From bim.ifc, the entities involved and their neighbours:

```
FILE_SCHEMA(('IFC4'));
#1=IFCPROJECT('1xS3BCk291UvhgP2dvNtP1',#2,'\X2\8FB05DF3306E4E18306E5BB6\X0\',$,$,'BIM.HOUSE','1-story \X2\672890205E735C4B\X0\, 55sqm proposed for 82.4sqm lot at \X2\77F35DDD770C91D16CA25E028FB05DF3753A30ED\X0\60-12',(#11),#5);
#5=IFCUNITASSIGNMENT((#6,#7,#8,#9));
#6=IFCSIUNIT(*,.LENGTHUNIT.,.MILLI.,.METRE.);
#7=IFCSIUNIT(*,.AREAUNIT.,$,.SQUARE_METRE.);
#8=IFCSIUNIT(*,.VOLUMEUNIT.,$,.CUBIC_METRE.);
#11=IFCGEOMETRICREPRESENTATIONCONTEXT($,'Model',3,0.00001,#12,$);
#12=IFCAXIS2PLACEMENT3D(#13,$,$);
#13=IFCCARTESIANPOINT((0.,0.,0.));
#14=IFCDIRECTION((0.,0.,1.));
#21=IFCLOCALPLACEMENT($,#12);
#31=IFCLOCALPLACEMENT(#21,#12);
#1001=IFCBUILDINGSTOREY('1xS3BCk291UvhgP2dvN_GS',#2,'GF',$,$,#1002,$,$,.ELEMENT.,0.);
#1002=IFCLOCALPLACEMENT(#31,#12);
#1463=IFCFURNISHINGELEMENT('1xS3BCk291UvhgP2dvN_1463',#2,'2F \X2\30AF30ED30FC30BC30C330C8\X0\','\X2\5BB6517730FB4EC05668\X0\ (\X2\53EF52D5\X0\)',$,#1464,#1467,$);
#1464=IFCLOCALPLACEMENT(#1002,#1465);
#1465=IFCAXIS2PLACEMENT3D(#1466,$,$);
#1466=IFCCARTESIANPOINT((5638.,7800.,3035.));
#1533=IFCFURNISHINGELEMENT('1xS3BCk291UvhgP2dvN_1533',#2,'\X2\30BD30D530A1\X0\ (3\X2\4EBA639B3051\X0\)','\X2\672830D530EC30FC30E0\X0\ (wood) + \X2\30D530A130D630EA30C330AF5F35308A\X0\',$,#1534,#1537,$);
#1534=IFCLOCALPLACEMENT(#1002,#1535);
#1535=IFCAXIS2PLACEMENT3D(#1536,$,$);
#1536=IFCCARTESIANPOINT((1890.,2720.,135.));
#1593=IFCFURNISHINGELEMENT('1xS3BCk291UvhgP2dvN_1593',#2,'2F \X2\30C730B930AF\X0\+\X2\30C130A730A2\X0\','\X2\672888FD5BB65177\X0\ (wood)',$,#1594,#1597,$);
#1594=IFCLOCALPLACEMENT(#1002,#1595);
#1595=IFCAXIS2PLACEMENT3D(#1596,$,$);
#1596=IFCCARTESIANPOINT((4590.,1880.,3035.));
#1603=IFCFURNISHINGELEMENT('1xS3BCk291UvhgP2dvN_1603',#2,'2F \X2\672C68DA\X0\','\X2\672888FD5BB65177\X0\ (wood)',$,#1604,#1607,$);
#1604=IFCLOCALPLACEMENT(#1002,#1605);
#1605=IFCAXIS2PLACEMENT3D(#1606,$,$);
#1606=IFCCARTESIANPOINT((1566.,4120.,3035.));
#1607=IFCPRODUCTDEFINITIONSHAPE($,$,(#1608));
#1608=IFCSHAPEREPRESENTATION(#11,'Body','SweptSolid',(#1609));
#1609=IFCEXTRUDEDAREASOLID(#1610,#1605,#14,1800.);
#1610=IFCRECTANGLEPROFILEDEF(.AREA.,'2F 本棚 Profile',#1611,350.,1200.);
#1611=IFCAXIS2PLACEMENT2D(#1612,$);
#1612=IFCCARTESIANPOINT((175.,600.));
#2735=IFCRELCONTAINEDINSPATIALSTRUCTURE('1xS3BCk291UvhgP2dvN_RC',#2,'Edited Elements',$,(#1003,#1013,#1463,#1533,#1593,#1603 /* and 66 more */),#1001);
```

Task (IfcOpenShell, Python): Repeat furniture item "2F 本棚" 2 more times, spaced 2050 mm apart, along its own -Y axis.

```python
import ifcopenshell
import ifcopenshell.api.geometry
import ifcopenshell.api.root
import ifcopenshell.util.element
import ifcopenshell.util.placement

model = ifcopenshell.open("bim.ifc")


def reuse_history(source, copy):
    """copy_class also copies each property set's owner history, people and application; keep the originals."""
    for rel in copy.IsDefinedBy:
        if rel.is_a("IfcRelDefinesByProperties") and (history := rel.RelatingPropertyDefinition.OwnerHistory):
            rel.RelatingPropertyDefinition.OwnerHistory = source.OwnerHistory
            ifcopenshell.util.element.remove_deep2(model, history)


source = model.by_guid("1xS3BCk291UvhgP2dvN_1603")
base = ifcopenshell.util.placement.get_local_placement(source.ObjectPlacement)
step = -base[:3, 1] * 2050.0

for i in range(1, 3):
    copy = ifcopenshell.api.root.copy_class(model, product=source)
    copy.Representation = ifcopenshell.util.element.copy_deep(
        model, source.Representation, exclude=["IfcGeometricRepresentationContext", "IfcRepresentationMap"]
    )
    reuse_history(source, copy)
    matrix = base.copy()
    matrix[:3, 3] += i * step
    print("added at", matrix[:3, 3].round(3) + 0.0)
    ifcopenshell.api.geometry.edit_object_placement(model, product=copy, matrix=matrix, is_si=False)

model.write("bim_rev.ifc")
```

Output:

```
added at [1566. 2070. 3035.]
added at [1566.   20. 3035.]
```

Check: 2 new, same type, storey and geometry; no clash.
